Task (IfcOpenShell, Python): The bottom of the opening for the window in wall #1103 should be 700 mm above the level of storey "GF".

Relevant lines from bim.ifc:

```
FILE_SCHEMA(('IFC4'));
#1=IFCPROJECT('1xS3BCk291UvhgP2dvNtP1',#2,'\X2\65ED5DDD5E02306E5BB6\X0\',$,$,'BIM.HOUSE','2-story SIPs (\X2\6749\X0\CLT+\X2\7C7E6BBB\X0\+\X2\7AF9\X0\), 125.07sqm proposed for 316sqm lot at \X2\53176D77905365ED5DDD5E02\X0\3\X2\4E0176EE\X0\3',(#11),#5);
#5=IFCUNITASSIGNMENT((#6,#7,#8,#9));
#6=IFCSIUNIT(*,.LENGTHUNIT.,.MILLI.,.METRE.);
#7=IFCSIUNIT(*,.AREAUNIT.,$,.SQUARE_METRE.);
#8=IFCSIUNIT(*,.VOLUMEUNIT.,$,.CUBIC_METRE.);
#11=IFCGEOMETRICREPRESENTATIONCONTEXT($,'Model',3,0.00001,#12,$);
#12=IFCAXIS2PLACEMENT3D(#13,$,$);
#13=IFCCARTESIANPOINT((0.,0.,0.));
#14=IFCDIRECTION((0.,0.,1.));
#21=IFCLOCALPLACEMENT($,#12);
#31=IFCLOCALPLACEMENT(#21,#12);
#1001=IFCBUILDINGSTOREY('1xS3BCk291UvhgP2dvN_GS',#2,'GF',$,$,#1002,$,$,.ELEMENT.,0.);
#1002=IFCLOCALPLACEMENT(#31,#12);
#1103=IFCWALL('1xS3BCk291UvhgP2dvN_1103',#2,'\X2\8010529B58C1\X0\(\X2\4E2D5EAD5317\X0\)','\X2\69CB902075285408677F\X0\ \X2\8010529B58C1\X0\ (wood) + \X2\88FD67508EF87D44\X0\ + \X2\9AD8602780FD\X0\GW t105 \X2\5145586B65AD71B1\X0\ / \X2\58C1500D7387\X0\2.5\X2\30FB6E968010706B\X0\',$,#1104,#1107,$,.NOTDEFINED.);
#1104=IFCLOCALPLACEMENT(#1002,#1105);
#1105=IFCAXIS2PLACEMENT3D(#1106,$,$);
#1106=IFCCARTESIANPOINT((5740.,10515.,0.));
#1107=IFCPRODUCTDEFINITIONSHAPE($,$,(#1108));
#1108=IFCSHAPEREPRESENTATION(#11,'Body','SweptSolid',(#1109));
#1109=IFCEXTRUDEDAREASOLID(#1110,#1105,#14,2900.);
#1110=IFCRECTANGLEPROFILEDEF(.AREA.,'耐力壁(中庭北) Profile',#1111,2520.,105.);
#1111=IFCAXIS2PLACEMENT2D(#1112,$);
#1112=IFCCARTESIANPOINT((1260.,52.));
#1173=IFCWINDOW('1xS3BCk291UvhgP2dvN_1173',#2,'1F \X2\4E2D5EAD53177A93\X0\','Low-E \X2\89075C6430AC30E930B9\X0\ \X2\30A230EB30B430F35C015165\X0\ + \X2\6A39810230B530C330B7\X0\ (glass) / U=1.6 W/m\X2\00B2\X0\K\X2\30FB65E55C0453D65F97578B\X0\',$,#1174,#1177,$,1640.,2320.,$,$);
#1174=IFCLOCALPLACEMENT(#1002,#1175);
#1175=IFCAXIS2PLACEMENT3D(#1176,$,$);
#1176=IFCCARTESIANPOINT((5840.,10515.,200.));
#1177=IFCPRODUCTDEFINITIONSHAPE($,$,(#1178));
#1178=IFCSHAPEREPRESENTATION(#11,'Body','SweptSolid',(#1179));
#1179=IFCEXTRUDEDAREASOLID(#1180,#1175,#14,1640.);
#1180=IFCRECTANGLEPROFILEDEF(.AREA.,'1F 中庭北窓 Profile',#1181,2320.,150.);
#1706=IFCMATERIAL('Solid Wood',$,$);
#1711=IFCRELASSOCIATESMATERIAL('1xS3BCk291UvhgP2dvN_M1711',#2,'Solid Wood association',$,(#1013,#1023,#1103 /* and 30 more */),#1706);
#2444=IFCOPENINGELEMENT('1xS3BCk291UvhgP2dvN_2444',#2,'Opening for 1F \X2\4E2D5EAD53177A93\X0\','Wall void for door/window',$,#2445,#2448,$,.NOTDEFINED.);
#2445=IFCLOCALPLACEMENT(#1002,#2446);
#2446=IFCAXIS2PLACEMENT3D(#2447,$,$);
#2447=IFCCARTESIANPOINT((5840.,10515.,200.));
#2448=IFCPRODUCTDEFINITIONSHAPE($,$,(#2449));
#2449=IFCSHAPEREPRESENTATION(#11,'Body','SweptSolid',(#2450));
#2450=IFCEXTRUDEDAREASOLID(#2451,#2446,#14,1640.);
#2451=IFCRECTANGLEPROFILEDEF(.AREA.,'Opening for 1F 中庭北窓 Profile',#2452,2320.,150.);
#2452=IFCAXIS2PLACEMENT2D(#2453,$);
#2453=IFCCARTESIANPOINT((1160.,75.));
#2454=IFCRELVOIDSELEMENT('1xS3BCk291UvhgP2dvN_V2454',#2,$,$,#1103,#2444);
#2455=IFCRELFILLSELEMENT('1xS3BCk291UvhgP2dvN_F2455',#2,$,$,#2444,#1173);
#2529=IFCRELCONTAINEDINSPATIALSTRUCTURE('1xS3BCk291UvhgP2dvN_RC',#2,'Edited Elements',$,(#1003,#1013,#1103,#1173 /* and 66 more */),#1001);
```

```python
import numpy as np
import ifcopenshell
import ifcopenshell.api.geometry
import ifcopenshell.geom
import ifcopenshell.util.element
import ifcopenshell.util.placement
import ifcopenshell.util.shape
import ifcopenshell.util.unit

model = ifcopenshell.open("bim.ifc")
unit_scale = ifcopenshell.util.unit.calculate_unit_scale(model)

window = model.by_guid("1xS3BCk291UvhgP2dvN_1173")
opening = window.FillsVoids[0].RelatingOpeningElement
storey = ifcopenshell.util.element.get_container(window, ifc_class="IfcBuildingStorey")
level = ifcopenshell.util.placement.get_local_placement(storey.ObjectPlacement)[2, 3]

# The opening's origin need not be at the sill, so measure its lowest point.
shape = ifcopenshell.geom.create_shape(ifcopenshell.geom.settings(), opening)
bottom = ifcopenshell.util.shape.get_shape_bottom_elevation(shape, shape.geometry) / unit_scale
dz = level + 0.7 / unit_scale - bottom

shift = np.array([0.0, 0.0, dz])
# The window is not placed relative to its opening, so move both.
for product in (opening, window):
    matrix = ifcopenshell.util.placement.get_local_placement(product.ObjectPlacement)
    matrix[:3, 3] += shift
    ifcopenshell.api.geometry.edit_object_placement(model, product=product, matrix=matrix, is_si=False)

print(f"moved by {dz * unit_scale:+.3f} m")

model.write("bim_v2.ifc")
```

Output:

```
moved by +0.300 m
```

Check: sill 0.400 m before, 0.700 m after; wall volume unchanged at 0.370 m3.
